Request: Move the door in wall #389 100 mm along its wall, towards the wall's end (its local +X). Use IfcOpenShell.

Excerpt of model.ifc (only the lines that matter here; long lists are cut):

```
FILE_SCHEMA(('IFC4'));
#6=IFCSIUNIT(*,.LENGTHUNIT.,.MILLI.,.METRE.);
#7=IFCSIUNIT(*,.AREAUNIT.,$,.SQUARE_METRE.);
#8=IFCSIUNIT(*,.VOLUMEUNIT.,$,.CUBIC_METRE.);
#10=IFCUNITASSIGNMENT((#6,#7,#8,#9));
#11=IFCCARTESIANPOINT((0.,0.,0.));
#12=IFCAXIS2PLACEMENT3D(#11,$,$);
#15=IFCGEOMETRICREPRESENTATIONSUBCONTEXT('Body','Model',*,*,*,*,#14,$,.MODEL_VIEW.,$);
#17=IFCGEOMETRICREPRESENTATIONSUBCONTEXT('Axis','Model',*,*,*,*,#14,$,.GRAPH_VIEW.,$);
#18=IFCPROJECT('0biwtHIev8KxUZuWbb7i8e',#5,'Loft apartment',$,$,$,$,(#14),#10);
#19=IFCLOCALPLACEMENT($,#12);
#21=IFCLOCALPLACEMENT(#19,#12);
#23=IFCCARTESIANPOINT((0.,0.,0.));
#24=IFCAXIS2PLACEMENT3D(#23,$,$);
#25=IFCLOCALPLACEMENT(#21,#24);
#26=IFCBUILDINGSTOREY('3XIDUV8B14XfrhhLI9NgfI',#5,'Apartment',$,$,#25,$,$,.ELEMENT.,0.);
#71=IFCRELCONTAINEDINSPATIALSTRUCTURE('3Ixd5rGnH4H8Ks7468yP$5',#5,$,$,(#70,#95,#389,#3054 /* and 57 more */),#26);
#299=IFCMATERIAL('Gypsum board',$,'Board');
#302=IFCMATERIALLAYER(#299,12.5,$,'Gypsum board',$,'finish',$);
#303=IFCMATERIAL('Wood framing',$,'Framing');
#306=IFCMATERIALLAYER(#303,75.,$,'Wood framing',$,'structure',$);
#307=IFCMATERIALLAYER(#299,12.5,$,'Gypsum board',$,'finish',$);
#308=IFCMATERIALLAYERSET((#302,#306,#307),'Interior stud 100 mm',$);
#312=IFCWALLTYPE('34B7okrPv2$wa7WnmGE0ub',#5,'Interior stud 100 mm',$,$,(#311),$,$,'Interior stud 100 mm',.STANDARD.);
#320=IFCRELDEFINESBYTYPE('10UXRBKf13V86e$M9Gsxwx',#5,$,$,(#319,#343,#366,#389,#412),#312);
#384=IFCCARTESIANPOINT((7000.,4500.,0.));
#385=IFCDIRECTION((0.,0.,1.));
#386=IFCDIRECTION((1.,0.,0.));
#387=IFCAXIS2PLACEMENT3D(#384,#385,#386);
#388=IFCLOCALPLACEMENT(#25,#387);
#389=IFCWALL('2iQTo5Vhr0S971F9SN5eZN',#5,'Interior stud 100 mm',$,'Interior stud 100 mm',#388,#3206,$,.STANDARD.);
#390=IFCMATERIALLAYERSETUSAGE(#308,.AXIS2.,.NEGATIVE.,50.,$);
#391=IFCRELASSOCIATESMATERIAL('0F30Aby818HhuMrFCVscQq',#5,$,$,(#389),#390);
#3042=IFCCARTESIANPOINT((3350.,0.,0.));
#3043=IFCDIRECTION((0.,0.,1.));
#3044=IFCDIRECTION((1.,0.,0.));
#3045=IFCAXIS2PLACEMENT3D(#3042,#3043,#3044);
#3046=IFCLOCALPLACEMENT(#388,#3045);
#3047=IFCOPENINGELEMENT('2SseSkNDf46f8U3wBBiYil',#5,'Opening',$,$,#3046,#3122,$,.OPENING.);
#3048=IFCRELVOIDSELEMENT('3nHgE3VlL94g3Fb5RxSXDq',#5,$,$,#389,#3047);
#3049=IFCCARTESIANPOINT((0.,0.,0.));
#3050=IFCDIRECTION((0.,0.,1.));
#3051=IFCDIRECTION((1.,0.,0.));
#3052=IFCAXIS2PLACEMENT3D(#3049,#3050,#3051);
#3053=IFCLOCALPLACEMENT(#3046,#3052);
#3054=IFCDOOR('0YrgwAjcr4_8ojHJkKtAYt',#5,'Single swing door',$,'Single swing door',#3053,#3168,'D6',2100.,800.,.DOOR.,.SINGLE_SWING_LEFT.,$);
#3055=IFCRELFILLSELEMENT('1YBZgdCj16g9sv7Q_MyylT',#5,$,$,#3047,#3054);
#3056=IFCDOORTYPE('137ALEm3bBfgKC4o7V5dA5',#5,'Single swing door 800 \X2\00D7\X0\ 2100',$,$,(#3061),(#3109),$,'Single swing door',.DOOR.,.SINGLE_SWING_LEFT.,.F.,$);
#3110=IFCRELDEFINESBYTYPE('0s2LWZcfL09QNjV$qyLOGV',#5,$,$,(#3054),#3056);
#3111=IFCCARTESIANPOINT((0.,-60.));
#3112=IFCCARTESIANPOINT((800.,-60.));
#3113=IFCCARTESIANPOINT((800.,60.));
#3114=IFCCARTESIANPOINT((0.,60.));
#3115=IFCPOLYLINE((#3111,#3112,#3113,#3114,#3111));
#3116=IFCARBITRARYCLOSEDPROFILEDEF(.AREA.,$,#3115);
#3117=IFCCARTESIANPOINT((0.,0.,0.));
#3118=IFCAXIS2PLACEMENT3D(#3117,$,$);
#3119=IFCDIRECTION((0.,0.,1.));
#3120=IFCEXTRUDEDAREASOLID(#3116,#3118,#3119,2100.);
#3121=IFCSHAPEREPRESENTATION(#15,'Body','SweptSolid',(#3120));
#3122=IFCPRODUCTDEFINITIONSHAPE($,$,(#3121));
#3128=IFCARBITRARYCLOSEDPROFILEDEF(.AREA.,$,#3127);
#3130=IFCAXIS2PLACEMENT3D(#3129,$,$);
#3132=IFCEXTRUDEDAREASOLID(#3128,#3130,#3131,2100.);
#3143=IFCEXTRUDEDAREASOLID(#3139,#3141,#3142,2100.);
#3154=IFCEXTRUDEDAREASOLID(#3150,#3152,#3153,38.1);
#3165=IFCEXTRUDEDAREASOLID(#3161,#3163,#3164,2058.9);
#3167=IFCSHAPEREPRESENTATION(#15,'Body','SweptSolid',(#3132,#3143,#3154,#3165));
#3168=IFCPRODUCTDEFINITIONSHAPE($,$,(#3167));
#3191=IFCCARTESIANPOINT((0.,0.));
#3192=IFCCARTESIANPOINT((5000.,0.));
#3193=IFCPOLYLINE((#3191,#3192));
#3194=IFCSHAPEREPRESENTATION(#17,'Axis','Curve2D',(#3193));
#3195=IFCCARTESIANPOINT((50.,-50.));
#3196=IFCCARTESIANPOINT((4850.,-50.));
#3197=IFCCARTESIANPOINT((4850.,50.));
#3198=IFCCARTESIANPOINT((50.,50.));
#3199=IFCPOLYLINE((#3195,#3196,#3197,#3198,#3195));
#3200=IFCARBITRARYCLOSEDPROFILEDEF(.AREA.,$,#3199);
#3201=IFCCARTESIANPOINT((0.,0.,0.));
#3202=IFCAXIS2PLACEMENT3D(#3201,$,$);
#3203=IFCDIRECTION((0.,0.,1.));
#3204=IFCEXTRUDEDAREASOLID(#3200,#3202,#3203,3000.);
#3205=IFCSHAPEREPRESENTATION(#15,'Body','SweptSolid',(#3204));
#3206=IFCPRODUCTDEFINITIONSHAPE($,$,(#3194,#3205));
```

```python
import ifcopenshell
import ifcopenshell.api.geometry
import ifcopenshell.util.placement
import ifcopenshell.util.unit

model = ifcopenshell.open("model.ifc")
unit_scale = ifcopenshell.util.unit.calculate_unit_scale(model)

door = model.by_guid("0YrgwAjcr4_8ojHJkKtAYt")
opening = door.FillsVoids[0].RelatingOpeningElement
wall = opening.VoidsElements[0].RelatingBuildingElement

wall_matrix = ifcopenshell.util.placement.get_local_placement(wall.ObjectPlacement)
shift = wall_matrix[:3, 0] * 0.1 / unit_scale
before = ifcopenshell.util.placement.get_local_placement(door.ObjectPlacement)[:3, 3].copy()

# The door is placed relative to its opening, so it follows when the opening moves.
matrix = ifcopenshell.util.placement.get_local_placement(opening.ObjectPlacement)
matrix[:3, 3] += shift
ifcopenshell.api.geometry.edit_object_placement(
    model, product=opening, matrix=matrix, is_si=False, should_transform_children=True
)

after = ifcopenshell.util.placement.get_local_placement(door.ObjectPlacement)[:3, 3]
print("door moved by", (after - before).round(3) + 0.0)

model.write("model_v2.ifc")
```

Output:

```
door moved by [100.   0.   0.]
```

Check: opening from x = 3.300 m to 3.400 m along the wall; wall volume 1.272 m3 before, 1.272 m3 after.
